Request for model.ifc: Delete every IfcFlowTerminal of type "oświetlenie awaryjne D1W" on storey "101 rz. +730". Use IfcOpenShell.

First a look at what the model holds.

```python
import ifcopenshell
import ifcopenshell.util.element

model = ifcopenshell.open("model.ifc")
print(model.schema)
storey = next(s for s in model.by_type("IfcBuildingStorey") if s.Name == "101 rz. +730")
terminals = [e for e in ifcopenshell.util.element.get_decomposition(storey) if e.is_a("IfcFlowTerminal")]
seen = {}
for e in terminals:
    element_type = ifcopenshell.util.element.get_type(e)
    name = element_type.Name if element_type not in (None, e) else None
    seen[name] = seen.get(name, 0) + 1
for name, count in sorted(seen.items(), key=str):
    print(count, "x", name)
```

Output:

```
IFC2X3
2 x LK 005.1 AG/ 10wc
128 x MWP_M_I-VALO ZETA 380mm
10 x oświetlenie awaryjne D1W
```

```python
import ifcopenshell
import ifcopenshell.api.root
import ifcopenshell.util.element

model = ifcopenshell.open("model.ifc")

storey = next(s for s in model.by_type("IfcBuildingStorey") if s.Name == "101 rz. +730")
terminals = [e for e in ifcopenshell.util.element.get_decomposition(storey) if e.is_a("IfcFlowTerminal")]
targets = [e for e in terminals if (t := ifcopenshell.util.element.get_type(e)) not in (None, e) and t.Name == "oświetlenie awaryjne D1W"]

for e in targets:
    ifcopenshell.api.root.remove_product(model, product=e)
print(len(targets), "removed")

model.write("model_updated.ifc")
```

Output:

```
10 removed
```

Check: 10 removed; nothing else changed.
